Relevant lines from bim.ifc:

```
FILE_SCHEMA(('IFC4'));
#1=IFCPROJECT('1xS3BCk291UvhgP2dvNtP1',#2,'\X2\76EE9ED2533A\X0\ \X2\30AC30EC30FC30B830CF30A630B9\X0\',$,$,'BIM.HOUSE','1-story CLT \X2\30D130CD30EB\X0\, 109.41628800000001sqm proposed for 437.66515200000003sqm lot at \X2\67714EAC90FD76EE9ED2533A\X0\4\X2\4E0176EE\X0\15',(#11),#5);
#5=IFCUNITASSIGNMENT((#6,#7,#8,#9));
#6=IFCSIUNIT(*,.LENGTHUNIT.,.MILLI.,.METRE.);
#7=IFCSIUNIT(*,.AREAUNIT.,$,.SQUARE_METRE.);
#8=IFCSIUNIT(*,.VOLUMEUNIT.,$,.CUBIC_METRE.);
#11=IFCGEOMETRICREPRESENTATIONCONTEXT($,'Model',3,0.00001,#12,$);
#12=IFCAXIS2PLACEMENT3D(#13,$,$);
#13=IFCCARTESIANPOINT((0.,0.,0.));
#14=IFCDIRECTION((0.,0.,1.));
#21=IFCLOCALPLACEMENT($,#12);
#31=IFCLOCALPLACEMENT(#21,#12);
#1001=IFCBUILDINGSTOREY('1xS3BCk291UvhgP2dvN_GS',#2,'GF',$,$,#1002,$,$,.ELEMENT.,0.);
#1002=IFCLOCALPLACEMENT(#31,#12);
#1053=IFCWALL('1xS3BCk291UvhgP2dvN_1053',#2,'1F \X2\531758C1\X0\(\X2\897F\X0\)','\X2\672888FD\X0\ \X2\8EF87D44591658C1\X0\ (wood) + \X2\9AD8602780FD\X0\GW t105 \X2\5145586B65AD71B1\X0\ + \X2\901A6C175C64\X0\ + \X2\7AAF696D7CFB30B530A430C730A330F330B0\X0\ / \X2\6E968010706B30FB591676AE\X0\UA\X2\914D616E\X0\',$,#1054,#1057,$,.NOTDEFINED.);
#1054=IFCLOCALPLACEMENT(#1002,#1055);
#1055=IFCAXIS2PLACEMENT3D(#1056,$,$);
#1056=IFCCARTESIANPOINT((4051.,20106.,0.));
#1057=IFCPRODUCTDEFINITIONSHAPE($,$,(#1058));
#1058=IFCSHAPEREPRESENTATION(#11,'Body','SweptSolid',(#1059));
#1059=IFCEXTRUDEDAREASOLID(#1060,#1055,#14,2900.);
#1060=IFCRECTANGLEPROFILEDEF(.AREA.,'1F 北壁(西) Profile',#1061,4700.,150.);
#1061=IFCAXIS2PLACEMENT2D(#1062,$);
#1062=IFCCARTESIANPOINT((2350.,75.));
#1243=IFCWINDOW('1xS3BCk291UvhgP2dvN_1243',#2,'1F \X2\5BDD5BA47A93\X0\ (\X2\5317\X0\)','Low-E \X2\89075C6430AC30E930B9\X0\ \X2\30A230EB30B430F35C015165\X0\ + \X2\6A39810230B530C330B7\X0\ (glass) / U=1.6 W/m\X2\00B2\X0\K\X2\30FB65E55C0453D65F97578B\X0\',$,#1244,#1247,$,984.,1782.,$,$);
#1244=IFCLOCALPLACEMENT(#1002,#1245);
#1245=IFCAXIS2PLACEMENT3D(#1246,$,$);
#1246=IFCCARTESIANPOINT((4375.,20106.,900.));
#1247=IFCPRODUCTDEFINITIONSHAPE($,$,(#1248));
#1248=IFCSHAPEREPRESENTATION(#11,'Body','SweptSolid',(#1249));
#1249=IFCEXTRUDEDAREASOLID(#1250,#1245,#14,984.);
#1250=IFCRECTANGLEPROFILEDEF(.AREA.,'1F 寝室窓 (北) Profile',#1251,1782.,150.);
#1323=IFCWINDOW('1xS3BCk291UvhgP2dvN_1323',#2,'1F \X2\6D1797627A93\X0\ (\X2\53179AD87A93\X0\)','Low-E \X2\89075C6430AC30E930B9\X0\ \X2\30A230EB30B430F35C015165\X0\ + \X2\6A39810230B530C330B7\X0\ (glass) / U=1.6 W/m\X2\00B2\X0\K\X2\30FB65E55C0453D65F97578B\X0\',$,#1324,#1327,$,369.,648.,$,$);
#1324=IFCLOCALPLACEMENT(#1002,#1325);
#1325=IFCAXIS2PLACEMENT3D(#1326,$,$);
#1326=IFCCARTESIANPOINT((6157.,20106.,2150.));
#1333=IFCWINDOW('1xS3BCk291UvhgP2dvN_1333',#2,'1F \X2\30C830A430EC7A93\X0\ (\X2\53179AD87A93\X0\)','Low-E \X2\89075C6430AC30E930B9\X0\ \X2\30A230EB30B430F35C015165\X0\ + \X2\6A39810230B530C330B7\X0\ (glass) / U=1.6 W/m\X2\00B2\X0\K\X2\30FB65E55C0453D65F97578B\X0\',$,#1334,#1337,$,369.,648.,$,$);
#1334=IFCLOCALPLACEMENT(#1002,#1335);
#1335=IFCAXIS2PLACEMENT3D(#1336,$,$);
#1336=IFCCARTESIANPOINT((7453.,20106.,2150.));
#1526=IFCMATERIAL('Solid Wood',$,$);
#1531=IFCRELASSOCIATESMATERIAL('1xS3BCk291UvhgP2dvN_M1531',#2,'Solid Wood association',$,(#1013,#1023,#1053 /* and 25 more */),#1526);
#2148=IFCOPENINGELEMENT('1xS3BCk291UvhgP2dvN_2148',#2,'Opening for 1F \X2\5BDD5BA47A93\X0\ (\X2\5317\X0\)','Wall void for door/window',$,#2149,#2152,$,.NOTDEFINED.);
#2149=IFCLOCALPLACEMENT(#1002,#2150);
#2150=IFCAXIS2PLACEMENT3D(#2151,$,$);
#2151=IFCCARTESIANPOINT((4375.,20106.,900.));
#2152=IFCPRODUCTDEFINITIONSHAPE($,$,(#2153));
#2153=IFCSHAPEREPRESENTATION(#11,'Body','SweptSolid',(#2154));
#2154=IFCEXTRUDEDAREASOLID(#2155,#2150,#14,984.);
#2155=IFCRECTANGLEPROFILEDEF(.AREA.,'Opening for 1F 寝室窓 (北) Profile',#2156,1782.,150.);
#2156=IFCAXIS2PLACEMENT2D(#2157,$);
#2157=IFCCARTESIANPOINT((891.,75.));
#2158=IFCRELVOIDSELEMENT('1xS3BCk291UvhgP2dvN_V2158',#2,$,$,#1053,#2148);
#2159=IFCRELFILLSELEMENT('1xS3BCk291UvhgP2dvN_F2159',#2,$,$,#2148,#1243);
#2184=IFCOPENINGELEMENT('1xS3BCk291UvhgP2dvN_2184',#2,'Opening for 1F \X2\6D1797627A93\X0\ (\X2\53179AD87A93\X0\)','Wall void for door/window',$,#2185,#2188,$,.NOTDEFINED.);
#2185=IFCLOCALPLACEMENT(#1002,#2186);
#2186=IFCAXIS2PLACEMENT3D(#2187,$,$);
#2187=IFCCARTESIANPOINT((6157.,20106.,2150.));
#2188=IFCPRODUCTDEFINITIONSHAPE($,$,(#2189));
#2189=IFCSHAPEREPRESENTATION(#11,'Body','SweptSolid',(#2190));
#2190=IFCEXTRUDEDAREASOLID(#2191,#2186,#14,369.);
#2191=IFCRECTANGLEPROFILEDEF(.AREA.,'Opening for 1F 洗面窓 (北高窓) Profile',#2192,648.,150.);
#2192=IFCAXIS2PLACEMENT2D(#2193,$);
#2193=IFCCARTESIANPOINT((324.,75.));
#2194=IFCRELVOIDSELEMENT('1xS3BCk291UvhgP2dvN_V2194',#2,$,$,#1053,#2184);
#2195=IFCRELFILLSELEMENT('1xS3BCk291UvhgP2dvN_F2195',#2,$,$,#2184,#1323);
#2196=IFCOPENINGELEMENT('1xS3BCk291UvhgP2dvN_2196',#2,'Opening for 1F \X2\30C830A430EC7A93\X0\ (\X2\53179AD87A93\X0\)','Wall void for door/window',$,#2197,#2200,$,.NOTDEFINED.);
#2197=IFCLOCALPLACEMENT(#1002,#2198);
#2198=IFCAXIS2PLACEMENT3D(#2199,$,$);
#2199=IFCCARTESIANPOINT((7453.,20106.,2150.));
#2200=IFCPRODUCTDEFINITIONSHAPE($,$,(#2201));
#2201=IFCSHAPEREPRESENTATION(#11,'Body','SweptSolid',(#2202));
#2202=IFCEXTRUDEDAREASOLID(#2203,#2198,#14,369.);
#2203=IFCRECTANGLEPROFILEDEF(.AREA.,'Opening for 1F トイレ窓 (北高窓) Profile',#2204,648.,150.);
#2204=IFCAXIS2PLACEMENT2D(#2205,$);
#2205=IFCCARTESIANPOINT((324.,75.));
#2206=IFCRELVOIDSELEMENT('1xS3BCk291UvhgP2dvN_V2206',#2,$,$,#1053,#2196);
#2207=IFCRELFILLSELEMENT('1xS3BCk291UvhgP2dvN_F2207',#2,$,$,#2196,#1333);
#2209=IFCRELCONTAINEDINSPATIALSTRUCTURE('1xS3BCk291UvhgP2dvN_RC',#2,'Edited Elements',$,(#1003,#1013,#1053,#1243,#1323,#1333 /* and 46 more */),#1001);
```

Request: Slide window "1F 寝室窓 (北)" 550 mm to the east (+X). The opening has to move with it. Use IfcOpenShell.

```python
import ifcopenshell
import ifcopenshell.api.geometry
import ifcopenshell.util.placement

model = ifcopenshell.open("bim.ifc")

window = model.by_guid("1xS3BCk291UvhgP2dvN_1243")
opening = window.FillsVoids[0].RelatingOpeningElement
wall = opening.VoidsElements[0].RelatingBuildingElement

wall_matrix = ifcopenshell.util.placement.get_local_placement(wall.ObjectPlacement)
shift = wall_matrix[:3, 0] * 550.0
before = ifcopenshell.util.placement.get_local_placement(window.ObjectPlacement)[:3, 3].copy()

# The window is not placed relative to its opening, so move both.
for product in (opening, window):
    matrix = ifcopenshell.util.placement.get_local_placement(product.ObjectPlacement)
    matrix[:3, 3] += shift
    ifcopenshell.api.geometry.edit_object_placement(model, product=product, matrix=matrix, is_si=False)

after = ifcopenshell.util.placement.get_local_placement(window.ObjectPlacement)[:3, 3]
print("window moved by", (after - before).round(3) + 0.0)

model.write("bim_edited.ifc")
```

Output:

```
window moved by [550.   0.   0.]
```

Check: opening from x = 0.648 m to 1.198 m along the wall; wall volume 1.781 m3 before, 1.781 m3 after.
